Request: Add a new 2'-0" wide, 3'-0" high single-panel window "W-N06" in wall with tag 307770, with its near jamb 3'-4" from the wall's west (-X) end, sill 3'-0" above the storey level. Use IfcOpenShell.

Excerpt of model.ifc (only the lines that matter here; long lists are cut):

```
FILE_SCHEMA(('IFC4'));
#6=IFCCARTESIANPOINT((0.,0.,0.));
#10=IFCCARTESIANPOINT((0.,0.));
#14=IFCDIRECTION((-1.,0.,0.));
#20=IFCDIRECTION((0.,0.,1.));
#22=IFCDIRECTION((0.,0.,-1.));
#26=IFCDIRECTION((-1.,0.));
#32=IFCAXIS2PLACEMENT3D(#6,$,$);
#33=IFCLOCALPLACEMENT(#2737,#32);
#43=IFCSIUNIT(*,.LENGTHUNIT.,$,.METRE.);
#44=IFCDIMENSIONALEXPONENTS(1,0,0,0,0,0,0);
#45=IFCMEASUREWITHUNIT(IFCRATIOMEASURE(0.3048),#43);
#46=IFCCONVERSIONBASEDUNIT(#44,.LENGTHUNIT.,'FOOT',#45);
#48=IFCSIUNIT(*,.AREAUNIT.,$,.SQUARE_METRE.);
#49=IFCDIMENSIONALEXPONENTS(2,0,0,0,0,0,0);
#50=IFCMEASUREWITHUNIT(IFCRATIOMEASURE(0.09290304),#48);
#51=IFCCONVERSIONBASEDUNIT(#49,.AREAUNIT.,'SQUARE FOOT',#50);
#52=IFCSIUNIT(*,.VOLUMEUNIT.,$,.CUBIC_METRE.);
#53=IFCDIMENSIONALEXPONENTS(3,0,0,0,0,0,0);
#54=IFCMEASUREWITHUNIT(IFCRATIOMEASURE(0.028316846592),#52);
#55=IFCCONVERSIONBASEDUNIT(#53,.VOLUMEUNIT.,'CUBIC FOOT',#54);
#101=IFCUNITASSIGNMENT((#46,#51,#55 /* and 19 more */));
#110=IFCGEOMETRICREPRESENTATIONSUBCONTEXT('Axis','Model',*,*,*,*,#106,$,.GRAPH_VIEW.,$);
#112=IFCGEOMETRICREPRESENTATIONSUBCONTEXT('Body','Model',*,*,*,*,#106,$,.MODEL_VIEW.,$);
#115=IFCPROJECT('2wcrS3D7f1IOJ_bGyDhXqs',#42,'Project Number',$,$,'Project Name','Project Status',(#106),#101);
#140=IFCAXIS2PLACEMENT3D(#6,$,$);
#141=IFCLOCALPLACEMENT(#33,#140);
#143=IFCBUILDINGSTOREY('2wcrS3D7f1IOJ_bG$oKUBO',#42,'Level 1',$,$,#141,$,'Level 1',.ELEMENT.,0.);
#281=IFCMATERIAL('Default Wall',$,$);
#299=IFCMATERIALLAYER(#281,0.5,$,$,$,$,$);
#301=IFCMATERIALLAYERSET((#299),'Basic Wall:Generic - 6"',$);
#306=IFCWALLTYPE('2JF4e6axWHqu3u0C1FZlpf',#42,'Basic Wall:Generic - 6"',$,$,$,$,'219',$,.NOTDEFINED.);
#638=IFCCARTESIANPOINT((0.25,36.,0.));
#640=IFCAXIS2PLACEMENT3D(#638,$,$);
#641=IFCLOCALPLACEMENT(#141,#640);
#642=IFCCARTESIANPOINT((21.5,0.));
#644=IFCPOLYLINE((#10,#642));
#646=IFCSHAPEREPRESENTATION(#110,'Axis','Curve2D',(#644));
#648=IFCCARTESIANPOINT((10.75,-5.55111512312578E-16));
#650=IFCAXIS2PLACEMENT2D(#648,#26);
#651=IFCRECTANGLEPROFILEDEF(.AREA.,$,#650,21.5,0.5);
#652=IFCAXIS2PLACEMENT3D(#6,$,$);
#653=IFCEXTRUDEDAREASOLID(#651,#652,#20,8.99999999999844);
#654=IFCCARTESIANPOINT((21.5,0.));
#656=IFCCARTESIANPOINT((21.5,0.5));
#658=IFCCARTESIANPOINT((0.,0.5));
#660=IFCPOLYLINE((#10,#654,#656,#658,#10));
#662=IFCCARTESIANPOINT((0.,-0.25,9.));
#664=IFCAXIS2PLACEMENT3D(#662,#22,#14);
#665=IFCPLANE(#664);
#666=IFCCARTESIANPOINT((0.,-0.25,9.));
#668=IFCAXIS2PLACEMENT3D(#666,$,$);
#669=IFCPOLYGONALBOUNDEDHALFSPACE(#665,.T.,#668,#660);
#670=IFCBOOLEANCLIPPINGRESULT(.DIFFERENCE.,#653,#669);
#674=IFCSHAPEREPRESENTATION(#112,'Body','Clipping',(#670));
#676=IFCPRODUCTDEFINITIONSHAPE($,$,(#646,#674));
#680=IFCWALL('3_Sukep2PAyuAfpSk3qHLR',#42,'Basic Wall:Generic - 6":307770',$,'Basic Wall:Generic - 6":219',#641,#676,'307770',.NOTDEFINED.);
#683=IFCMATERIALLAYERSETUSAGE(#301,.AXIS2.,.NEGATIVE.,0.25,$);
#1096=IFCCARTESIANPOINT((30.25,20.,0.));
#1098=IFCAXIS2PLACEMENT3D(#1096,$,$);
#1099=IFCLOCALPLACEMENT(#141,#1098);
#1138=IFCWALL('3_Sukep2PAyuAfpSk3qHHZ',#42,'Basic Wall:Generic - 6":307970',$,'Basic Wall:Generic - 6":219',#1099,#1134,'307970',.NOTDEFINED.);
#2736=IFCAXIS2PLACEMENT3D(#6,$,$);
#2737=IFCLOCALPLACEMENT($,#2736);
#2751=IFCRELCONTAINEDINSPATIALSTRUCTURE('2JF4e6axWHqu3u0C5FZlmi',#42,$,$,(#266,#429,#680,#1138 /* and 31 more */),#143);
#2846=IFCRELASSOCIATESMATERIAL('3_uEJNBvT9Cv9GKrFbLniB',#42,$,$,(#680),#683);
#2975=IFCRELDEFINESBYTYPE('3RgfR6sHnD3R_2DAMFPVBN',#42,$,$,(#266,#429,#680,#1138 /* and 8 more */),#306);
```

```python
import numpy as np
import ifcopenshell
import ifcopenshell.api.feature
import ifcopenshell.api.geometry
import ifcopenshell.api.root
import ifcopenshell.api.spatial
import ifcopenshell.geom
import ifcopenshell.util.element
import ifcopenshell.util.placement
import ifcopenshell.util.representation
import ifcopenshell.util.shape
import ifcopenshell.util.unit

model = ifcopenshell.open("model.ifc")
unit_scale = ifcopenshell.util.unit.calculate_unit_scale(model)
settings = ifcopenshell.geom.settings()


def volume(element):
    """Net volume in cubic metres, openings subtracted."""
    shape = ifcopenshell.geom.create_shape(settings, element)
    return ifcopenshell.util.shape.get_volume(shape.geometry)


wall = model.by_id(680)
storey = ifcopenshell.util.element.get_container(wall, ifc_class="IfcBuildingStorey")
context = ifcopenshell.util.representation.get_context(model, "Model", "Body", "MODEL_VIEW")
before = volume(wall)

width, height, from_end, sill = 0.6096, 0.9144, 1.016, 0.9144  # metres

# The wall runs along its own X axis, and the end named is its -X end.
wall_shape = ifcopenshell.geom.create_shape(settings, wall)
x, y, z = ifcopenshell.util.shape.get_vertices(wall_shape.geometry).T
start = x.min() + from_end
face, thickness = float(y.min()), float(y.max() - y.min())
wall_matrix = ifcopenshell.util.placement.get_local_placement(wall.ObjectPlacement)
level = ifcopenshell.util.placement.get_local_placement(storey.ObjectPlacement)[2, 3]


def in_wall(x, y):
    """Placement at x, y metres in the wall's axes, at sill height."""
    matrix = wall_matrix.copy()
    matrix[:, 3] = wall_matrix @ np.array([x / unit_scale, y / unit_scale, 0.0, 1.0])
    matrix[2, 3] = level + sill / unit_scale
    return matrix


# Opening: a box that overshoots both wall faces by 50 mm.
opening = ifcopenshell.api.root.create_entity(model, ifc_class="IfcOpeningElement", predefined_type="OPENING")
box = ifcopenshell.api.geometry.add_wall_representation(
    model, context=context, length=width, height=height, thickness=thickness + 0.1
)
ifcopenshell.api.geometry.assign_representation(model, product=opening, representation=box)
ifcopenshell.api.geometry.edit_object_placement(model, product=opening, matrix=in_wall(start, face - 0.05), is_si=False)
ifcopenshell.api.feature.add_feature(model, feature=opening, element=wall)

window = ifcopenshell.api.root.create_entity(model, ifc_class="IfcWindow", name="W-N06", predefined_type="WINDOW")
window.OverallWidth, window.OverallHeight = width / unit_scale, height / unit_scale
window.PartitioningType = "SINGLE_PANEL"
body = ifcopenshell.api.geometry.add_window_representation(
    model,
    context=context,
    overall_width=window.OverallWidth,
    overall_height=window.OverallHeight,
    partition_type="SINGLE_PANEL",
)
ifcopenshell.api.geometry.assign_representation(model, product=window, representation=body)
ifcopenshell.api.spatial.assign_container(model, products=[window], relating_structure=storey)
ifcopenshell.api.feature.add_filling(model, opening=opening, element=window)

# Centre the window in the wall's thickness.
ifcopenshell.api.geometry.edit_object_placement(model, product=window, matrix=in_wall(start, face), is_si=False)
window_shape = ifcopenshell.geom.create_shape(settings, window)
depth = ifcopenshell.util.shape.get_vertices(window_shape.geometry)[:, 1]
offset = face + thickness / 2 - (depth.min() + depth.max()) / 2
ifcopenshell.api.geometry.edit_object_placement(model, product=window, matrix=in_wall(start, offset), is_si=False)

after = volume(wall)

print(f"wall volume {before:.3f} -> {after:.3f} m3")

model.write("model_v2.ifc")
```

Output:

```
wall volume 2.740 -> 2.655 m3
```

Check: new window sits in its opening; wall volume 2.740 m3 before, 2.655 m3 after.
